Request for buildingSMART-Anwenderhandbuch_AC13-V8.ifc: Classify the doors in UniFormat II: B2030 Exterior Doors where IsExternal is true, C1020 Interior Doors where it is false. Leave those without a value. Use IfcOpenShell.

First a look at what the model holds.

```python
import ifcopenshell
import ifcopenshell.util.element

model = ifcopenshell.open("buildingSMART-Anwenderhandbuch_AC13-V8.ifc")
print(model.schema)
print("classifications:", [c.Name for c in model.by_type("IfcClassification")])
values = [ifcopenshell.util.element.get_pset(e, "Pset_DoorCommon", "IsExternal") for e in model.by_type("IfcDoor")]
for value in (True, False, None):
    print("IsExternal", value, values.count(value))
```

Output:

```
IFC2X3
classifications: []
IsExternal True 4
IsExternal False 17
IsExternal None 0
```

```python
import ifcopenshell
import ifcopenshell.api.classification
import ifcopenshell.util.element

model = ifcopenshell.open("buildingSMART-Anwenderhandbuch_AC13-V8.ifc")

# IFC2X3 requires Source and Edition and has no link from the project to the system.
system = model.create_entity("IfcClassification", Source="ASTM", Edition="E1557", Name="UniFormat II")

doors = model.by_type("IfcDoor")
external = {e: ifcopenshell.util.element.get_pset(e, "Pset_DoorCommon", "IsExternal") for e in doors}
for flag, code, name in ((True, "B2030", "Exterior Doors"), (False, "C1020", "Interior Doors")):
    products = [e for e in doors if external[e] is flag]
    ifcopenshell.api.classification.add_reference(
        model, products=products, classification=system, identification=code, name=name
    )
    print(code, len(products))

model.write("buildingSMART-Anwenderhandbuch_AC13-V8-out.ifc")
```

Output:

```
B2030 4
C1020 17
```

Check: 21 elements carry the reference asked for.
